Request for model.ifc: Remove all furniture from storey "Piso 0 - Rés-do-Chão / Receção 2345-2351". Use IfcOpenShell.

First a look at what the model holds.

```python
import ifcopenshell
import ifcopenshell.util.element

model = ifcopenshell.open("model.ifc")
print(model.schema)
storey = next(s for s in model.by_type("IfcBuildingStorey") if s.Name == "Piso 0 - Rés-do-Chão / Receção 2345-2351")
furniture = [e for e in ifcopenshell.util.element.get_decomposition(storey) if e.is_a("IfcFurnishingElement")]
seen = {}
for e in furniture:
    element_type = ifcopenshell.util.element.get_type(e)
    name = element_type.Name if element_type not in (None, e) else None
    seen[name] = seen.get(name, 0) + 1
for name, count in sorted(seen.items(), key=str):
    print(count, "x", name)
```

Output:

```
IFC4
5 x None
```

```python
import ifcopenshell
import ifcopenshell.api.root
import ifcopenshell.util.element

model = ifcopenshell.open("model.ifc")

storey = next(s for s in model.by_type("IfcBuildingStorey") if s.Name == "Piso 0 - Rés-do-Chão / Receção 2345-2351")
furniture = [e for e in ifcopenshell.util.element.get_decomposition(storey) if e.is_a("IfcFurnishingElement")]

for e in furniture:
    ifcopenshell.api.root.remove_product(model, product=e)
print(len(furniture), "removed")

model.write("model_edited.ifc")
```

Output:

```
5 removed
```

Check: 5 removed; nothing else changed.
